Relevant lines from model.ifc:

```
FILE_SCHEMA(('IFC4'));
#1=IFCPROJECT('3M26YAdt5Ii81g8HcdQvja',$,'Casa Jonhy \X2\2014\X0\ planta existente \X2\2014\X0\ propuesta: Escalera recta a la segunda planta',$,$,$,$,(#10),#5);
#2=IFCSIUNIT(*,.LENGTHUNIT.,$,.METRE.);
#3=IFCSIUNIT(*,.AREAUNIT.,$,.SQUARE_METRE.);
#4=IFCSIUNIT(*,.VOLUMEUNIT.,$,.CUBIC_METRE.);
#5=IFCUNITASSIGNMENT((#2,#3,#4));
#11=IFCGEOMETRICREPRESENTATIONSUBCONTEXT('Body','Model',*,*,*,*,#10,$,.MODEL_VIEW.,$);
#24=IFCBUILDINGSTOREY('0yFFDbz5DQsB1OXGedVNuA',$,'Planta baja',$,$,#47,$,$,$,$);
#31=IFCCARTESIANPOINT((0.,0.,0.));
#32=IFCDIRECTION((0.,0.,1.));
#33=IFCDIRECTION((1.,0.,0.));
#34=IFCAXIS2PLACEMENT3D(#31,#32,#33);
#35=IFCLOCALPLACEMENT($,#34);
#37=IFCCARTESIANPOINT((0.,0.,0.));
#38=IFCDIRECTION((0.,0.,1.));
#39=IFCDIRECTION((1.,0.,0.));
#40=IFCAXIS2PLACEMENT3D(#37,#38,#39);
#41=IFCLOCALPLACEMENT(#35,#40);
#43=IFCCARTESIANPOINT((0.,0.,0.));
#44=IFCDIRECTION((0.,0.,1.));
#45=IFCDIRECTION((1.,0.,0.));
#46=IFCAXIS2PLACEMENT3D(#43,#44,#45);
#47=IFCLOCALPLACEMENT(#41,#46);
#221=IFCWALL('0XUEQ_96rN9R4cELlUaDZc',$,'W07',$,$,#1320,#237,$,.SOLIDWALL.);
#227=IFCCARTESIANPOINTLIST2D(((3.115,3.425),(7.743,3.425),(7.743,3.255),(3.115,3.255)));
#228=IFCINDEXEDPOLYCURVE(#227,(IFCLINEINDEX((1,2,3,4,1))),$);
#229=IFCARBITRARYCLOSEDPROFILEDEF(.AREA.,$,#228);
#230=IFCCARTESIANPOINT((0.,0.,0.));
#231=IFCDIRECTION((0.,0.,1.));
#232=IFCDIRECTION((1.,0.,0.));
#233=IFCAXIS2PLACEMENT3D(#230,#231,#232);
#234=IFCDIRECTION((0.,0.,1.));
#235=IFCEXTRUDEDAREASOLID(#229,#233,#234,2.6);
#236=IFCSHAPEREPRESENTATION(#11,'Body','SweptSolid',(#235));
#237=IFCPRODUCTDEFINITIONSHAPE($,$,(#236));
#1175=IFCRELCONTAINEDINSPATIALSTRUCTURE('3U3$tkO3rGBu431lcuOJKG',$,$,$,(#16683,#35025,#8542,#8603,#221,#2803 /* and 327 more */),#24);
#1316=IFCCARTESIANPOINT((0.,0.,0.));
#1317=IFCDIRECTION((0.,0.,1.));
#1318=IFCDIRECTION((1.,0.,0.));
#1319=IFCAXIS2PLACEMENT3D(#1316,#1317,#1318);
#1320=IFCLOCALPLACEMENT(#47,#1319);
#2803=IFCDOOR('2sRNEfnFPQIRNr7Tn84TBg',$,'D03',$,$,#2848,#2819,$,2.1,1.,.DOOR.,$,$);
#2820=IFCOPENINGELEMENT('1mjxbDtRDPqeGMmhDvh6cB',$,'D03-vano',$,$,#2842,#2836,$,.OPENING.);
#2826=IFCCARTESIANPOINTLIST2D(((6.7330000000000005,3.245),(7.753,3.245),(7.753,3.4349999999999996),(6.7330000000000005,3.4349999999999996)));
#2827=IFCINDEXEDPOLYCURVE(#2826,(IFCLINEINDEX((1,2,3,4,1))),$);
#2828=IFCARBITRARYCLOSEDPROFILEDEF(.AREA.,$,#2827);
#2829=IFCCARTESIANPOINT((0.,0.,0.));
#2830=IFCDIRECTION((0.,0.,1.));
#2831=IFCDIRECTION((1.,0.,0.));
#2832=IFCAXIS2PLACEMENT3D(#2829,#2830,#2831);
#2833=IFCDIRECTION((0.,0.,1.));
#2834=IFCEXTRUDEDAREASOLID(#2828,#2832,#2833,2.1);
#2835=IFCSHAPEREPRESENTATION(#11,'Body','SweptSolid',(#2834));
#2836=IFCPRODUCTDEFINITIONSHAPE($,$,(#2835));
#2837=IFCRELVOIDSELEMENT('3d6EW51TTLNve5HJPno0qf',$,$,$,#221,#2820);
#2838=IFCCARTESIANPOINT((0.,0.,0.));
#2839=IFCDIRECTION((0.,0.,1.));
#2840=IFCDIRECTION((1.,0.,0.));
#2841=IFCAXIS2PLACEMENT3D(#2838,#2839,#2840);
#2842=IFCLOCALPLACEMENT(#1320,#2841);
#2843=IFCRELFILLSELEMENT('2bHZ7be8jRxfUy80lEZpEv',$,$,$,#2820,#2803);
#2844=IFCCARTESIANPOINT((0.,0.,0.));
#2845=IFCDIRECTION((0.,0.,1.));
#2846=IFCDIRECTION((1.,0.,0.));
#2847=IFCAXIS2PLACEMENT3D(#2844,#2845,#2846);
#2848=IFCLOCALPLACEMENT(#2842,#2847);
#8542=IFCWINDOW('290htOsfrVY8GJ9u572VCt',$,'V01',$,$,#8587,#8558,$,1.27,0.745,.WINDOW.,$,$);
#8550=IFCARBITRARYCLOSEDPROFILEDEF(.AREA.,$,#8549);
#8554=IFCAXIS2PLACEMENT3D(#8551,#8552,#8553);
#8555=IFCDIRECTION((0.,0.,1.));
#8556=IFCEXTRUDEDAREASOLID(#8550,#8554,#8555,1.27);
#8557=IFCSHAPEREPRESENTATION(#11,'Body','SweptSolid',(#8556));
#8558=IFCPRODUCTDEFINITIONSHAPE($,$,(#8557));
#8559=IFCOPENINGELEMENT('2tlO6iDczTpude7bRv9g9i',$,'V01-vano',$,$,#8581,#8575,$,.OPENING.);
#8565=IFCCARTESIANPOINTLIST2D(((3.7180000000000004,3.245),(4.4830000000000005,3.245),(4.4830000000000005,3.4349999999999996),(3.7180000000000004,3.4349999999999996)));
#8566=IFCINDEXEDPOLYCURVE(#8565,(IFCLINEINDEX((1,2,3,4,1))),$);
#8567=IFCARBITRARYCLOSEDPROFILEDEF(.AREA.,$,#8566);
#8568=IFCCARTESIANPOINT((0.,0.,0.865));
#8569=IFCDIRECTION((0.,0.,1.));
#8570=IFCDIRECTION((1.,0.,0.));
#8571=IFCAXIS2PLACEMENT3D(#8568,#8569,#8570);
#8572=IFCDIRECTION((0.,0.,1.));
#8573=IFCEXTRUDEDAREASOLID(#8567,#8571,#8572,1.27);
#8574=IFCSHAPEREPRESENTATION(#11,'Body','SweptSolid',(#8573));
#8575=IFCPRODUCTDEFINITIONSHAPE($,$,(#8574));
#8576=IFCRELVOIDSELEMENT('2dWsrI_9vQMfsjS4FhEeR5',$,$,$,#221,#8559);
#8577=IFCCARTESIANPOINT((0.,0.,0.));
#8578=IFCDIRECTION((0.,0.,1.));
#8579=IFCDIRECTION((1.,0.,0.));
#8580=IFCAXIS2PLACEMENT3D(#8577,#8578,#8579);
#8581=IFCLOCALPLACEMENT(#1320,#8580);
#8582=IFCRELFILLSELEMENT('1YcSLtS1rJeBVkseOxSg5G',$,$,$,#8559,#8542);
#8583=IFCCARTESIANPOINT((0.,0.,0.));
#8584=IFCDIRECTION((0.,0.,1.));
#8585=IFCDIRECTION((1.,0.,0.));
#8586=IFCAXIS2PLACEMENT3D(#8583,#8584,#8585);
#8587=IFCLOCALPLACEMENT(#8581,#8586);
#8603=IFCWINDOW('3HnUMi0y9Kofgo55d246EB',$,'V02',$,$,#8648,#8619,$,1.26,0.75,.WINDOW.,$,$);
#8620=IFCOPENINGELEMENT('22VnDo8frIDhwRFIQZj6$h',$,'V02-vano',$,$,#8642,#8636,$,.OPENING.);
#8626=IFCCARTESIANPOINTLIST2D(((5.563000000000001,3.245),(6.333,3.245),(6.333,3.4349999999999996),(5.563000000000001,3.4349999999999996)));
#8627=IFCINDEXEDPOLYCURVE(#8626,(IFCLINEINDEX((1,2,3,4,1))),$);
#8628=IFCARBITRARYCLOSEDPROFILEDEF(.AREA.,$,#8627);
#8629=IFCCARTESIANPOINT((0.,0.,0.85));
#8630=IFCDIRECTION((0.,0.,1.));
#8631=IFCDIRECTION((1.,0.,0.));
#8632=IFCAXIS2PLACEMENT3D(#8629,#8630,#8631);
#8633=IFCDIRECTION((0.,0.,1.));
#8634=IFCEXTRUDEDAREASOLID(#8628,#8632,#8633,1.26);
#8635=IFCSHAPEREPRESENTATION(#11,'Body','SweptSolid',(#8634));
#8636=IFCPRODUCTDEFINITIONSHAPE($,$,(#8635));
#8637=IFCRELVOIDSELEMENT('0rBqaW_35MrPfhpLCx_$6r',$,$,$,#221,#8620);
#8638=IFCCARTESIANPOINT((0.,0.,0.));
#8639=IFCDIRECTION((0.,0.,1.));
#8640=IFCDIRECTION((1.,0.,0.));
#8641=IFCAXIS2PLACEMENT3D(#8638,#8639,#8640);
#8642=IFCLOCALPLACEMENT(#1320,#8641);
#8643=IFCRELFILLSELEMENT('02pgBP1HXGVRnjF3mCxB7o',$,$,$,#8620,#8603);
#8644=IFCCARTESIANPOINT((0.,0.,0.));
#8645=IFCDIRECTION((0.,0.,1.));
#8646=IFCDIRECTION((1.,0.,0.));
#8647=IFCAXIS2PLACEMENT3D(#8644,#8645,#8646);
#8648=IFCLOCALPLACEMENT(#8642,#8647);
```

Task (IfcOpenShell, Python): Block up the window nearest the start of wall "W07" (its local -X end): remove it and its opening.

```python
import ifcopenshell
import ifcopenshell.api.feature
import ifcopenshell.api.root
import ifcopenshell.geom
import ifcopenshell.util.shape

model = ifcopenshell.open("model.ifc")
settings = ifcopenshell.geom.settings()


def volume(element):
    """Net volume in cubic metres, openings subtracted."""
    shape = ifcopenshell.geom.create_shape(settings, element)
    return ifcopenshell.util.shape.get_volume(shape.geometry)


window = model.by_guid("290htOsfrVY8GJ9u572VCt")
opening = window.FillsVoids[0].RelatingOpeningElement
wall = opening.VoidsElements[0].RelatingBuildingElement
before = volume(wall)

ifcopenshell.api.root.remove_product(model, product=window)
ifcopenshell.api.feature.remove_feature(model, feature=opening)

after = volume(wall)

print(f"wall volume {before:.3f} -> {after:.3f} m3")

model.write("model_rev.ifc")
```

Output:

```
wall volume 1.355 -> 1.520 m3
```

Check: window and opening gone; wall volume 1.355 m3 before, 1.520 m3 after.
